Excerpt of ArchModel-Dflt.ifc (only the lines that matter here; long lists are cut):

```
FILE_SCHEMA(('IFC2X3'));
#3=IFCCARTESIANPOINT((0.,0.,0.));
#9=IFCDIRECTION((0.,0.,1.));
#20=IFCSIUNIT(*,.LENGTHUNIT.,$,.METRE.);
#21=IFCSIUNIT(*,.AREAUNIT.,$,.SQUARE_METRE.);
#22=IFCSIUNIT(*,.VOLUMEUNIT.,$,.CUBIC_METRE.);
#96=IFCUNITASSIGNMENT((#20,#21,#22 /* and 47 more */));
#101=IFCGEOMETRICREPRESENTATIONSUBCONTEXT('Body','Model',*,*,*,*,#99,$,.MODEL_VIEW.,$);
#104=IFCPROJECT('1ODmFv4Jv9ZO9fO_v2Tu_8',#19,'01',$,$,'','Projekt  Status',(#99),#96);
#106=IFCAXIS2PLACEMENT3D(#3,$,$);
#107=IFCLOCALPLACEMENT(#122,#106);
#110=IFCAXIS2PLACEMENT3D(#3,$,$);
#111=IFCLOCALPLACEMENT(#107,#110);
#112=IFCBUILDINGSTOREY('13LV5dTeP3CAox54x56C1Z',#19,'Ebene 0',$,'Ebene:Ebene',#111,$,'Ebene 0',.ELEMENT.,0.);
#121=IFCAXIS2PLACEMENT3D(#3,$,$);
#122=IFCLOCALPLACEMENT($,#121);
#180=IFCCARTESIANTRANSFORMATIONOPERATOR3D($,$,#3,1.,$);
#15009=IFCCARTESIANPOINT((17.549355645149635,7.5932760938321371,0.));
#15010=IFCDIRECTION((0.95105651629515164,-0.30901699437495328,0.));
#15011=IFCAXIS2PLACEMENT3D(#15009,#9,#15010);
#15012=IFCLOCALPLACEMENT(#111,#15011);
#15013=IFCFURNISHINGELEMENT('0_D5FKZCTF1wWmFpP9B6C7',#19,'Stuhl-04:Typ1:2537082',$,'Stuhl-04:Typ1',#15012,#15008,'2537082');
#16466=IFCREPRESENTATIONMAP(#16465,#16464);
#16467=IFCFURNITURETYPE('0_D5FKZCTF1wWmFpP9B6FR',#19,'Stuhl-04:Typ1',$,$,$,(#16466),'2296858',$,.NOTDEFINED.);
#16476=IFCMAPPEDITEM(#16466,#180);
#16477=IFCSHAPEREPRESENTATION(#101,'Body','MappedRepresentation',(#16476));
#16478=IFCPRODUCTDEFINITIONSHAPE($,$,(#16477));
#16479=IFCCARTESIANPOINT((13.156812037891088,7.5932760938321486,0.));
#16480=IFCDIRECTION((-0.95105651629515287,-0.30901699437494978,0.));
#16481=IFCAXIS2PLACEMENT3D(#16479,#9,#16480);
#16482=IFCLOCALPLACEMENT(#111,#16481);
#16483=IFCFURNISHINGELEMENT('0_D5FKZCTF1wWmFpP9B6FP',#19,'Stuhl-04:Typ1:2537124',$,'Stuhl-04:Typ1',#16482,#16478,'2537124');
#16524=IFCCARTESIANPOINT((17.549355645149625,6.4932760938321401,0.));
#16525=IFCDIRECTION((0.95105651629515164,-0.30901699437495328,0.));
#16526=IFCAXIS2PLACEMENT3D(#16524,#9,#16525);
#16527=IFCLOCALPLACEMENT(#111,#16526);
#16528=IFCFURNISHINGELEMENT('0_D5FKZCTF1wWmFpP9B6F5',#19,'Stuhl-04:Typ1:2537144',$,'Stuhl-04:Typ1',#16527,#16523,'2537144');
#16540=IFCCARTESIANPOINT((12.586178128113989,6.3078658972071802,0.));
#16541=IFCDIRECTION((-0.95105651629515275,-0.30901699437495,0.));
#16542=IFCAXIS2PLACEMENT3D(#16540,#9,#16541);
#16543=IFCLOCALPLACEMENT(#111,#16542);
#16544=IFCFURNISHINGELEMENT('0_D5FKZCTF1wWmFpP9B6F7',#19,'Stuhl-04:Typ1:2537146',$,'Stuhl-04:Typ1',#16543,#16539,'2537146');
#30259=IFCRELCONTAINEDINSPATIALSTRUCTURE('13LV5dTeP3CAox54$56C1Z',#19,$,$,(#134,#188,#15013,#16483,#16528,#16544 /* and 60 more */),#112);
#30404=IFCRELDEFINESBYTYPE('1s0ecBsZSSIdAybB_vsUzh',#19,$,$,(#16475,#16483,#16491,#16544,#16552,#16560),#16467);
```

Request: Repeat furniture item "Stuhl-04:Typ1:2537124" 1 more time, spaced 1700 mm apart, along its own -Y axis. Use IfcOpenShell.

```python
import ifcopenshell
import ifcopenshell.api.geometry
import ifcopenshell.api.root
import ifcopenshell.util.element
import ifcopenshell.util.placement
import ifcopenshell.util.unit

model = ifcopenshell.open("ArchModel-Dflt.ifc")
unit_scale = ifcopenshell.util.unit.calculate_unit_scale(model)

source = model.by_id(16483)
base = ifcopenshell.util.placement.get_local_placement(source.ObjectPlacement)
step = -base[:3, 1] * 1.7 / unit_scale

for i in range(1, 2):
    copy = ifcopenshell.api.root.copy_class(model, product=source)
    copy.Representation = ifcopenshell.util.element.copy_deep(
        model, source.Representation, exclude=["IfcGeometricRepresentationContext", "IfcRepresentationMap"]
    )
    copy.Name = "Stuhl-04:Typ1"
    copy.Tag = None
    matrix = base.copy()
    matrix[:3, 3] += i * step
    print("added at", matrix[:3, 3].round(3) + 0.0)
    ifcopenshell.api.geometry.edit_object_placement(model, product=copy, matrix=matrix, is_si=False)

model.write("ArchModel-Dflt_v2.ifc")
```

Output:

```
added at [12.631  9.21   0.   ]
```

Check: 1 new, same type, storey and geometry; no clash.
